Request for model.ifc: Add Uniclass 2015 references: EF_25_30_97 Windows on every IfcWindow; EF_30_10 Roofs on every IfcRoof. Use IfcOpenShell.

First a look at what the model holds.

```python
import ifcopenshell

model = ifcopenshell.open("model.ifc")
print(model.schema)
print("classifications:", [c.Name for c in model.by_type("IfcClassification")])
for ifc_class in ("IfcDoor", "IfcRoof", "IfcStair", "IfcWall", "IfcWindow"):
    print(ifc_class, len(model.by_type(ifc_class)))
```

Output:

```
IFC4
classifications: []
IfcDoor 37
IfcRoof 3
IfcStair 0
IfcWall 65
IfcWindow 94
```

```python
import ifcopenshell
import ifcopenshell.api.classification

model = ifcopenshell.open("model.ifc")

system = ifcopenshell.api.classification.add_classification(model, classification="Uniclass 2015")

codes = {
    "IfcWindow": ("EF_25_30_97", "Windows"),
    "IfcRoof": ("EF_30_10", "Roofs"),
}
for ifc_class, (code, name) in codes.items():
    products = model.by_type(ifc_class)
    ifcopenshell.api.classification.add_reference(
        model, products=products, classification=system, identification=code, name=name
    )
    print(code, len(products))

model.write("model_v2.ifc")
```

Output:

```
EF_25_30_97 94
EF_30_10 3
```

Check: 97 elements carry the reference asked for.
